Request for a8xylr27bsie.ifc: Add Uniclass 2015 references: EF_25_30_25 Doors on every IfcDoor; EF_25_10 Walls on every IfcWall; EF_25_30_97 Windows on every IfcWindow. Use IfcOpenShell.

First a look at what the model holds.

```python
import ifcopenshell

model = ifcopenshell.open("a8xylr27bsie.ifc")
print(model.schema)
print("classifications:", [c.Name for c in model.by_type("IfcClassification")])
for ifc_class in ("IfcDoor", "IfcRoof", "IfcStair", "IfcWall", "IfcWindow"):
    print(ifc_class, len(model.by_type(ifc_class)))
```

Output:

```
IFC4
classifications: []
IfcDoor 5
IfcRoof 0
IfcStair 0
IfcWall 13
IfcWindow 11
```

```python
import ifcopenshell
import ifcopenshell.api.classification

model = ifcopenshell.open("a8xylr27bsie.ifc")

system = ifcopenshell.api.classification.add_classification(model, classification="Uniclass 2015")

codes = {
    "IfcDoor": ("EF_25_30_25", "Doors"),
    "IfcWall": ("EF_25_10", "Walls"),
    "IfcWindow": ("EF_25_30_97", "Windows"),
}
for ifc_class, (code, name) in codes.items():
    products = model.by_type(ifc_class)
    ifcopenshell.api.classification.add_reference(
        model, products=products, classification=system, identification=code, name=name
    )
    print(code, len(products))

model.write("a8xylr27bsie_v2.ifc")
```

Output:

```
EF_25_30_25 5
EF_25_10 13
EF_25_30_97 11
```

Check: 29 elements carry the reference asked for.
